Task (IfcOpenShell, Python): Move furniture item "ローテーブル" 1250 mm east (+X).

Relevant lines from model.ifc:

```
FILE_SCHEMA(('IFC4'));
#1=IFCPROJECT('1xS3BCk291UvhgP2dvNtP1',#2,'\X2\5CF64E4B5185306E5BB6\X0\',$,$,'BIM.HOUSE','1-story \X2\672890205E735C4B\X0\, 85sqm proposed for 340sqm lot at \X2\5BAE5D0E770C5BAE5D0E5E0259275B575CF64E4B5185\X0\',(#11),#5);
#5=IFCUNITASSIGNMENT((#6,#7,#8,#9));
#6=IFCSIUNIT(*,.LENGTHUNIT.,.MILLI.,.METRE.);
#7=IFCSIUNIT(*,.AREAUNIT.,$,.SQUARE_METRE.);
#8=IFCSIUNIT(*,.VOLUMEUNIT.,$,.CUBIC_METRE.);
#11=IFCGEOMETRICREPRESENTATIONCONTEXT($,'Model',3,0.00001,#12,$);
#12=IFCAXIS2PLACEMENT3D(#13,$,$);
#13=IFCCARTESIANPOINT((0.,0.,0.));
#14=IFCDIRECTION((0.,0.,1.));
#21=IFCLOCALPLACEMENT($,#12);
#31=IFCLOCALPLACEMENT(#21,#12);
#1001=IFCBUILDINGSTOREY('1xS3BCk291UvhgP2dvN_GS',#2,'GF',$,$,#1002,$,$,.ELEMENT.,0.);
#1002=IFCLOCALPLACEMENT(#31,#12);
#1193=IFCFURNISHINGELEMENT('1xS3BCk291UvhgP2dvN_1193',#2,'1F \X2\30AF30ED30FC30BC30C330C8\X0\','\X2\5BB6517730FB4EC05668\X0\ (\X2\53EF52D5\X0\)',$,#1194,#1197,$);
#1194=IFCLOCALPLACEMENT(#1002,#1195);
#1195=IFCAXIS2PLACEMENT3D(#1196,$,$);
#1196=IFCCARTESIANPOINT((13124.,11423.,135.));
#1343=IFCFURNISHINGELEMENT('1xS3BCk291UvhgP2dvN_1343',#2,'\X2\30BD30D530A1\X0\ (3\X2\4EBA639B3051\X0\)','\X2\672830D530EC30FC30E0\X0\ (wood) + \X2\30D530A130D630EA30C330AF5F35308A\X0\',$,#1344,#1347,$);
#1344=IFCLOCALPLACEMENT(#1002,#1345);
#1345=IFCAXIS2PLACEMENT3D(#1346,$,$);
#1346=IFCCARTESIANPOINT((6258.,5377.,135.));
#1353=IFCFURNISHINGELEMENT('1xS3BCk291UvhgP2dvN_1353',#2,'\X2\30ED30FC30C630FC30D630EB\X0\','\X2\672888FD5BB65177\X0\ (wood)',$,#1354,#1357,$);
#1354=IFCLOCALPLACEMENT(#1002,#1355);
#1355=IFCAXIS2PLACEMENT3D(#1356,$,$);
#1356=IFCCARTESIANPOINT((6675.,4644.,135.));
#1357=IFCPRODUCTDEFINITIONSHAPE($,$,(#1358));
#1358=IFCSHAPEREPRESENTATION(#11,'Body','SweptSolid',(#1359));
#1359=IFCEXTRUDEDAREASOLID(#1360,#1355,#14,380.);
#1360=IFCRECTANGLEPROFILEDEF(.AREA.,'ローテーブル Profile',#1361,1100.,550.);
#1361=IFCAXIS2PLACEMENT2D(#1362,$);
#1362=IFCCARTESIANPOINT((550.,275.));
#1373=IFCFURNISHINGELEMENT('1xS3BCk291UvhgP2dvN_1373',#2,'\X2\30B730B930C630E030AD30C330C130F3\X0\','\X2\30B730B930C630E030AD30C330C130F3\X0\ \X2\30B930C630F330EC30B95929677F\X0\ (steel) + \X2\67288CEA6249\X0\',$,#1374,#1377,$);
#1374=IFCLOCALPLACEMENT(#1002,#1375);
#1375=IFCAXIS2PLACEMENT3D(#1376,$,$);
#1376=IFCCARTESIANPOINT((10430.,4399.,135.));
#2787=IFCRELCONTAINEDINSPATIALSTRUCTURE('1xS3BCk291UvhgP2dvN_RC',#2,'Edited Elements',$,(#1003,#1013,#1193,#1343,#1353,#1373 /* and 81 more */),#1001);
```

```python
import ifcopenshell
import ifcopenshell.api.geometry
import ifcopenshell.util.placement
import ifcopenshell.util.unit

model = ifcopenshell.open("model.ifc")
unit_scale = ifcopenshell.util.unit.calculate_unit_scale(model)

item = model.by_guid("1xS3BCk291UvhgP2dvN_1353")
matrix = ifcopenshell.util.placement.get_local_placement(item.ObjectPlacement)
matrix[0, 3] += 1.25 / unit_scale
ifcopenshell.api.geometry.edit_object_placement(model, product=item, matrix=matrix, is_si=False)

print(ifcopenshell.util.placement.get_local_placement(item.ObjectPlacement).round(3) + 0.0)

model.write("model-out.ifc")
```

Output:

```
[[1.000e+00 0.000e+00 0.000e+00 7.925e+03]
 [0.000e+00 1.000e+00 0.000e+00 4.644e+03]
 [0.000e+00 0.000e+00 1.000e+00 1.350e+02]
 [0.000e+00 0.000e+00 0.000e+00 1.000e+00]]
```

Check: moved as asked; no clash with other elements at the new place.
